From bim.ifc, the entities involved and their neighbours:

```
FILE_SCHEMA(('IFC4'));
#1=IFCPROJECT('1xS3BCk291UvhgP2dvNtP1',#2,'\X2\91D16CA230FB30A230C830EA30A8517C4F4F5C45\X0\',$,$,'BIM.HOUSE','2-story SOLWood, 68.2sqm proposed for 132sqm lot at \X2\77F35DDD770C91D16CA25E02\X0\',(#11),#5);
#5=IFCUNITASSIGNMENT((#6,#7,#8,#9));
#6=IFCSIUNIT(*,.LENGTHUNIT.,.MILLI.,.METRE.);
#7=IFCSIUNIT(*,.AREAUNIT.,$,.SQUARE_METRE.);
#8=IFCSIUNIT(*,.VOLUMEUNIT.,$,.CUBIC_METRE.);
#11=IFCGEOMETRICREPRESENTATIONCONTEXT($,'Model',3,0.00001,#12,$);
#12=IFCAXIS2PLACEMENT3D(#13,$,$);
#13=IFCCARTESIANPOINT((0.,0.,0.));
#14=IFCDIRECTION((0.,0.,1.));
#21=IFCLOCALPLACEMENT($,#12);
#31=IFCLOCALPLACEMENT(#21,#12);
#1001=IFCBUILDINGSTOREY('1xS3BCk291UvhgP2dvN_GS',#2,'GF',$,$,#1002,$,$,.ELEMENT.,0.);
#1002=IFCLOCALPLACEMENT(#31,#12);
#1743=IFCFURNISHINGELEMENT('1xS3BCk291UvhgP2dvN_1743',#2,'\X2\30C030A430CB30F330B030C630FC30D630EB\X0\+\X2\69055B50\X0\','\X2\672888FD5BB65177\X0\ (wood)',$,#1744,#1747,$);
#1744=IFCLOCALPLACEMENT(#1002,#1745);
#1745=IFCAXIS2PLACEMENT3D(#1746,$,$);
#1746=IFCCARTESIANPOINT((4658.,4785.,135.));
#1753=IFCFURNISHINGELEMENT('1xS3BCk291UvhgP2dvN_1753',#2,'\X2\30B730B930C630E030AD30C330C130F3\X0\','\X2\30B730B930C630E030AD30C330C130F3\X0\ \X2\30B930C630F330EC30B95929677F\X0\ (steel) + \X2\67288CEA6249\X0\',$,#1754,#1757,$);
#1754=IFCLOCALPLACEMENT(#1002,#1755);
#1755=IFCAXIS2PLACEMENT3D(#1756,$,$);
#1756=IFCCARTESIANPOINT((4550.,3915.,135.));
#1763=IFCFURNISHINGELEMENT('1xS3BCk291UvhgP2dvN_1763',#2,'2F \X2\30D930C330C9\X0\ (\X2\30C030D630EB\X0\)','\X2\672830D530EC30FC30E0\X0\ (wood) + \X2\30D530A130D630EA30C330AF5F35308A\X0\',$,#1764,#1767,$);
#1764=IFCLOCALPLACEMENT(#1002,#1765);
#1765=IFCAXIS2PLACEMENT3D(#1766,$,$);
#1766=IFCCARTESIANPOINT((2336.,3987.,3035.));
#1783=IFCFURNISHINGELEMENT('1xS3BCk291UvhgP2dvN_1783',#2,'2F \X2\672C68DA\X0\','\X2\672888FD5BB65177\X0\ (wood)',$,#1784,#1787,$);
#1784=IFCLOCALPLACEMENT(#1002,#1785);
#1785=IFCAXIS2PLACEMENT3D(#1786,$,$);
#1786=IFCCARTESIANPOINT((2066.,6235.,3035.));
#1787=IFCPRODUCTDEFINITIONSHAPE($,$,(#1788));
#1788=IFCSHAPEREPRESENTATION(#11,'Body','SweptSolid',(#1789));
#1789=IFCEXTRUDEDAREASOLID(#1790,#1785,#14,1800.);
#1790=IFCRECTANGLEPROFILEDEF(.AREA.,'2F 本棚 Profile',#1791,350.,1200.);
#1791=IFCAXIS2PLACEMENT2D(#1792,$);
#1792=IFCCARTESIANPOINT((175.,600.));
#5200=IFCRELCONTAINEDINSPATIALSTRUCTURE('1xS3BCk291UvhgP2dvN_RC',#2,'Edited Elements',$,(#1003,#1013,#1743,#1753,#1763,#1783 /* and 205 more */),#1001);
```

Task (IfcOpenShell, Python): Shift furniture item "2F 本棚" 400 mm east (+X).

```python
import ifcopenshell
import ifcopenshell.api.geometry
import ifcopenshell.util.placement
import ifcopenshell.util.unit

model = ifcopenshell.open("bim.ifc")
unit_scale = ifcopenshell.util.unit.calculate_unit_scale(model)

item = model.by_guid("1xS3BCk291UvhgP2dvN_1783")
matrix = ifcopenshell.util.placement.get_local_placement(item.ObjectPlacement)
matrix[0, 3] += 0.4 / unit_scale
ifcopenshell.api.geometry.edit_object_placement(model, product=item, matrix=matrix, is_si=False)

print(ifcopenshell.util.placement.get_local_placement(item.ObjectPlacement).round(3) + 0.0)

model.write("bim_v2.ifc")
```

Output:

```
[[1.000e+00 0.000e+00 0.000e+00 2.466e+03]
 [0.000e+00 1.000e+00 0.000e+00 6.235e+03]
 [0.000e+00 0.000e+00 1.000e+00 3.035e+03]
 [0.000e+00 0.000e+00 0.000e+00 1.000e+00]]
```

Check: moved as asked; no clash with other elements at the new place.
